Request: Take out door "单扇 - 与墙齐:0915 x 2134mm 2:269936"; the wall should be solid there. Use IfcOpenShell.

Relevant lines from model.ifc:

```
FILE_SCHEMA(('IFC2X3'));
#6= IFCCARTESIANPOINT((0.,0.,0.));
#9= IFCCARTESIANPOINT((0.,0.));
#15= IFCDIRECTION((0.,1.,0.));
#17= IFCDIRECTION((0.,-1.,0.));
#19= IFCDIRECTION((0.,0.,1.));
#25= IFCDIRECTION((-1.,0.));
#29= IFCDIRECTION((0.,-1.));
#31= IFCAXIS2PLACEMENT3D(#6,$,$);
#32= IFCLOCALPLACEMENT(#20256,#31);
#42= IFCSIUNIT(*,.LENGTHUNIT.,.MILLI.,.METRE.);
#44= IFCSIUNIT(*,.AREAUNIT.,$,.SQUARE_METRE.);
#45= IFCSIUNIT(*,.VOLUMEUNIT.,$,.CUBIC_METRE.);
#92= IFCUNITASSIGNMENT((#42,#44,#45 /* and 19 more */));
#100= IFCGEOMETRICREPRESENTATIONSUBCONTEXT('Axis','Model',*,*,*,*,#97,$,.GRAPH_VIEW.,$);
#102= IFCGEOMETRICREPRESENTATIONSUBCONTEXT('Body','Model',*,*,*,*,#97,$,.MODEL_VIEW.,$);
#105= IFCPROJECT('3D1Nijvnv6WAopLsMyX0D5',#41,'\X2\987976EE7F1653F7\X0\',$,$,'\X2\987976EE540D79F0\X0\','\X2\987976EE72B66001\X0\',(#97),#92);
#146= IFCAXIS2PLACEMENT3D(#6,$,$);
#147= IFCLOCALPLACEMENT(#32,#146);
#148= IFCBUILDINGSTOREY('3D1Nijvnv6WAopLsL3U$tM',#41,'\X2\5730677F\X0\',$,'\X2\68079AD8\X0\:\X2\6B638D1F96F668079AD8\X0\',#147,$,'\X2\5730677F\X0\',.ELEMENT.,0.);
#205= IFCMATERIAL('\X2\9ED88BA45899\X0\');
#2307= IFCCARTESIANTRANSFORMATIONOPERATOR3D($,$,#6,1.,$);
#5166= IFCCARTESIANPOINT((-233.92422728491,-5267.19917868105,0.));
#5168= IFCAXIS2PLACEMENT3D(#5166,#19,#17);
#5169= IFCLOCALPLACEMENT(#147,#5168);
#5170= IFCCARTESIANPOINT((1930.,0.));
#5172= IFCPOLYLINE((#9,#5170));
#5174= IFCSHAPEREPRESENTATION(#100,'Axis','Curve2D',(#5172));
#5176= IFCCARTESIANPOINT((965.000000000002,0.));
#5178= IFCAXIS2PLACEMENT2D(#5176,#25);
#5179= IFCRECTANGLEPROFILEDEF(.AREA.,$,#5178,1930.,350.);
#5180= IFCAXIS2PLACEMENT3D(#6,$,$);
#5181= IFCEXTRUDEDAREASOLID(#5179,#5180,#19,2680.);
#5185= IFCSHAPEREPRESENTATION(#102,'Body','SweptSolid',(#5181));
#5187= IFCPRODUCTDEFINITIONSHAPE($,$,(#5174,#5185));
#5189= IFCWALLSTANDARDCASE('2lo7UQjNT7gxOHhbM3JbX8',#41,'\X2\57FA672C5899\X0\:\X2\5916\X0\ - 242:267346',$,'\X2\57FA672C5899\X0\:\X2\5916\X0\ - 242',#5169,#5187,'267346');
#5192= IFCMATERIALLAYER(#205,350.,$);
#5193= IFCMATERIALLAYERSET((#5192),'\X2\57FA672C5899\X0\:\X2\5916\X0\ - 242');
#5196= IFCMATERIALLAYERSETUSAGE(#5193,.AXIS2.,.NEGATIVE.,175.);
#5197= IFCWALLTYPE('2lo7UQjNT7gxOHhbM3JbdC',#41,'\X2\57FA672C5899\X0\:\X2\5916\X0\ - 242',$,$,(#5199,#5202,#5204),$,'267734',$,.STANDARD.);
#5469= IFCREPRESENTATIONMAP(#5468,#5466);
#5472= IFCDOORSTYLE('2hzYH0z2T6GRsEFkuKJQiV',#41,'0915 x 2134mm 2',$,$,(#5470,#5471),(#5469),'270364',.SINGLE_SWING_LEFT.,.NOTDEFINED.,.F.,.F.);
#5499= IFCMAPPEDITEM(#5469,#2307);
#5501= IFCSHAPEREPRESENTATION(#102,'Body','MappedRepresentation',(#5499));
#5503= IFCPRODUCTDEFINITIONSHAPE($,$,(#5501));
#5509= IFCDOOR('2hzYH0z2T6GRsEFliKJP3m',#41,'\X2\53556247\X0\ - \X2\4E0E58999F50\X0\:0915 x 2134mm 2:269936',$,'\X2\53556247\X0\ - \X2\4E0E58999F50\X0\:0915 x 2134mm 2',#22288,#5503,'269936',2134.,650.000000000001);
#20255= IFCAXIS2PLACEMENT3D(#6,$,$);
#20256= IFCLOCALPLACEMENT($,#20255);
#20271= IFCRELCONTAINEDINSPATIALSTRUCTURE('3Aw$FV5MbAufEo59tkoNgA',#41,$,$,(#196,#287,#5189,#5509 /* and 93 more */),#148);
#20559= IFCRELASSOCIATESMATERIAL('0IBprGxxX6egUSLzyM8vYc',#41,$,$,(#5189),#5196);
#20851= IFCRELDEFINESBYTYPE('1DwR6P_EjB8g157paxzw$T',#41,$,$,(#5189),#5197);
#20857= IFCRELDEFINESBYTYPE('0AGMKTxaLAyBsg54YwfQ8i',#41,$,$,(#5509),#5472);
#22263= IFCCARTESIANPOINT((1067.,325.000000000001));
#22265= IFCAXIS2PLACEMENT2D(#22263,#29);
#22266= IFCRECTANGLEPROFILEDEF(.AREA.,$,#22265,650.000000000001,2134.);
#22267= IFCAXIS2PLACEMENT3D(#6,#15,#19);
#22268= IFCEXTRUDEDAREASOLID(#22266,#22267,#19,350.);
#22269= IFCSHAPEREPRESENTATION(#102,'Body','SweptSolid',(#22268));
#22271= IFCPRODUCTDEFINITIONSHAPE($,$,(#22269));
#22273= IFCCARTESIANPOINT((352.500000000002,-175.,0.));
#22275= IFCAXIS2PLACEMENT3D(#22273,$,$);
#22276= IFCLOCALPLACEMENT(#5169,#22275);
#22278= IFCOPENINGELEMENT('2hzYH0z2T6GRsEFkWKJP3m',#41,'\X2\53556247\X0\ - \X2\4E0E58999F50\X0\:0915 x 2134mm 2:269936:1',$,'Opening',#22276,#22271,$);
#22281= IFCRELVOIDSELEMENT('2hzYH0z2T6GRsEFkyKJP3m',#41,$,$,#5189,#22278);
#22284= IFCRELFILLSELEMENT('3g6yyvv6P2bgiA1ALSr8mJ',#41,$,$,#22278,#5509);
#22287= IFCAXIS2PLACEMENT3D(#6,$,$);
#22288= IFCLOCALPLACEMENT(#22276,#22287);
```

```python
import ifcopenshell
import ifcopenshell.api.feature
import ifcopenshell.api.root
import ifcopenshell.geom
import ifcopenshell.util.shape

model = ifcopenshell.open("model.ifc")
settings = ifcopenshell.geom.settings()


def volume(element):
    """Net volume in cubic metres, openings subtracted."""
    shape = ifcopenshell.geom.create_shape(settings, element)
    return ifcopenshell.util.shape.get_volume(shape.geometry)


door = model.by_guid("2hzYH0z2T6GRsEFliKJP3m")
opening = door.FillsVoids[0].RelatingOpeningElement
wall = opening.VoidsElements[0].RelatingBuildingElement
before = volume(wall)

ifcopenshell.api.root.remove_product(model, product=door)
ifcopenshell.api.feature.remove_feature(model, feature=opening)

after = volume(wall)

print(f"wall volume {before:.3f} -> {after:.3f} m3")

model.write("model_v2.ifc")
```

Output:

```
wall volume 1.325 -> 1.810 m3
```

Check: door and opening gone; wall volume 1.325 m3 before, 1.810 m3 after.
